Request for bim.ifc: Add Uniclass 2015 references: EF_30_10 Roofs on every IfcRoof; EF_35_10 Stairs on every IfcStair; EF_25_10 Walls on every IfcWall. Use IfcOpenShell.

First a look at what the model holds.

```python
import ifcopenshell

model = ifcopenshell.open("bim.ifc")
print(model.schema)
print("classifications:", [c.Name for c in model.by_type("IfcClassification")])
for ifc_class in ("IfcDoor", "IfcRoof", "IfcStair", "IfcWall", "IfcWindow"):
    print(ifc_class, len(model.by_type(ifc_class)))
```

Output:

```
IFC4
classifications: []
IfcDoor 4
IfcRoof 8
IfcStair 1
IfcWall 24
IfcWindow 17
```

```python
import ifcopenshell
import ifcopenshell.api.classification

model = ifcopenshell.open("bim.ifc")

system = ifcopenshell.api.classification.add_classification(model, classification="Uniclass 2015")

codes = {
    "IfcRoof": ("EF_30_10", "Roofs"),
    "IfcStair": ("EF_35_10", "Stairs"),
    "IfcWall": ("EF_25_10", "Walls"),
}
for ifc_class, (code, name) in codes.items():
    products = model.by_type(ifc_class)
    ifcopenshell.api.classification.add_reference(
        model, products=products, classification=system, identification=code, name=name
    )
    print(code, len(products))

model.write("bim_edited.ifc")
```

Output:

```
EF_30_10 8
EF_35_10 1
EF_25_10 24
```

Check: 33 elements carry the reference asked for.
